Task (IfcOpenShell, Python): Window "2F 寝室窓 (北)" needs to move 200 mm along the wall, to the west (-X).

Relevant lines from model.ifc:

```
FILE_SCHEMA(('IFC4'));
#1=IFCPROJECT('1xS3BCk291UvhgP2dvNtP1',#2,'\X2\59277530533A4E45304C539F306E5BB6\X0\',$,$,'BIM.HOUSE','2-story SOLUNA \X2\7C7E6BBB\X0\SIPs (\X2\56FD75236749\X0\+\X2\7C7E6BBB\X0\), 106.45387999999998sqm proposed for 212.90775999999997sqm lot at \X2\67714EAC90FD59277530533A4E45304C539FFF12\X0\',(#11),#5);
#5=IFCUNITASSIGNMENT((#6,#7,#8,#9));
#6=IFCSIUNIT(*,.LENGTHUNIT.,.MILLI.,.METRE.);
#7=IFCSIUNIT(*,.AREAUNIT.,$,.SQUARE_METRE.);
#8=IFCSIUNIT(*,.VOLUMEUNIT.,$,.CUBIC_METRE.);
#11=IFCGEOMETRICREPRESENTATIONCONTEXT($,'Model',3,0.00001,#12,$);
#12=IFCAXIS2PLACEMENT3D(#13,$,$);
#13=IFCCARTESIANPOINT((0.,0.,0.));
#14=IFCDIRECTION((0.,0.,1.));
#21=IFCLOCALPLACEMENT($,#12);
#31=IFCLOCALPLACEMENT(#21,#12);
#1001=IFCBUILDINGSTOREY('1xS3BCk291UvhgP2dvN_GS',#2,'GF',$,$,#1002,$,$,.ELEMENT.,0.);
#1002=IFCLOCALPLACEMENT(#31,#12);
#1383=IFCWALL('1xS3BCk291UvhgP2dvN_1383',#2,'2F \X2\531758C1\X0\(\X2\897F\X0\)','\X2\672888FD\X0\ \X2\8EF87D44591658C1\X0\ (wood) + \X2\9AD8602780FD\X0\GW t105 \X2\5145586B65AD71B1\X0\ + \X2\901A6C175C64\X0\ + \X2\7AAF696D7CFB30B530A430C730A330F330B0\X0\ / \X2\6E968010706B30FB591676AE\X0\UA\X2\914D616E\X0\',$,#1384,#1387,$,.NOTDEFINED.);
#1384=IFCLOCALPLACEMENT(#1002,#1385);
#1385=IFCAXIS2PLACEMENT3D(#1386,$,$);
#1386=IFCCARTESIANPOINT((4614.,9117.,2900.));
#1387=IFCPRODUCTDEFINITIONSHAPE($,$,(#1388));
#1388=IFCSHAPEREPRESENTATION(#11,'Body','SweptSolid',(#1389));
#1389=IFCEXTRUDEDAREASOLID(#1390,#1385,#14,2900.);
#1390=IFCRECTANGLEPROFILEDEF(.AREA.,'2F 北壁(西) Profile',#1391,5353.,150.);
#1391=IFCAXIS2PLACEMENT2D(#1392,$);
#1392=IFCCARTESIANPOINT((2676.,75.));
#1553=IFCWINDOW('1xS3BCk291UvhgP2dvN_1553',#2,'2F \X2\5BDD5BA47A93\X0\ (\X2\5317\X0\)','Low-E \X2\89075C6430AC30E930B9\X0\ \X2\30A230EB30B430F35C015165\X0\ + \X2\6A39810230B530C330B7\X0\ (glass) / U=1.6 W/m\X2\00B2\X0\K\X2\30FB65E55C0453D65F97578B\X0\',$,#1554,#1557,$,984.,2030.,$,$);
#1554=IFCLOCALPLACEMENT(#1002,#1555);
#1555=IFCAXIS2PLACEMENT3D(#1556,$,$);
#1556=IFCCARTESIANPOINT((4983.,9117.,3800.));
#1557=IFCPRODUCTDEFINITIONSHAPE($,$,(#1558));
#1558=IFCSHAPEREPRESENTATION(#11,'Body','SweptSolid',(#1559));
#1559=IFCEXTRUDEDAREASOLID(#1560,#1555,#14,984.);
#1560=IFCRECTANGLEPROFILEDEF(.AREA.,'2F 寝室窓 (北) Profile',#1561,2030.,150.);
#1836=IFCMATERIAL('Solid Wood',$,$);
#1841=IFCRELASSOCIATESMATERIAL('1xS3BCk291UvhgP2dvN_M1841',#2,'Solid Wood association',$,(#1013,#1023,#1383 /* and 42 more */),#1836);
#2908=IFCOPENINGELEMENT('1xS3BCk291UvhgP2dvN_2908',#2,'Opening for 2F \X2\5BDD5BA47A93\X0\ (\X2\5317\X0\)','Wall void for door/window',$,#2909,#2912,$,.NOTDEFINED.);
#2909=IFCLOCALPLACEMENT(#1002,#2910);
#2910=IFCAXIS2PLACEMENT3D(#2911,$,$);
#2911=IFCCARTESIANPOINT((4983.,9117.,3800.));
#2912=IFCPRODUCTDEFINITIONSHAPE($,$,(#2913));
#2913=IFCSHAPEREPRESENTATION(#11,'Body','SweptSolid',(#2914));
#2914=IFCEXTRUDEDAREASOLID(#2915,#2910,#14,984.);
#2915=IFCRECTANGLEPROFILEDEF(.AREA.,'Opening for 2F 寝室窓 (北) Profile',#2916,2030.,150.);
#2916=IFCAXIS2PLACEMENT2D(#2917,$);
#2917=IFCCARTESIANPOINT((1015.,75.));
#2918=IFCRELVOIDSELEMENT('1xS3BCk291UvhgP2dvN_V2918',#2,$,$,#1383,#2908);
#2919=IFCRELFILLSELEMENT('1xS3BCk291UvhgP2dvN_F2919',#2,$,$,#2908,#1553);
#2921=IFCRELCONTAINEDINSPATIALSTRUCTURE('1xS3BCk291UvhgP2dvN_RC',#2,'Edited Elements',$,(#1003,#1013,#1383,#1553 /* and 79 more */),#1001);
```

```python
import ifcopenshell
import ifcopenshell.api.geometry
import ifcopenshell.util.placement
import ifcopenshell.util.unit

model = ifcopenshell.open("model.ifc")
unit_scale = ifcopenshell.util.unit.calculate_unit_scale(model)

window = model.by_guid("1xS3BCk291UvhgP2dvN_1553")
opening = window.FillsVoids[0].RelatingOpeningElement
wall = opening.VoidsElements[0].RelatingBuildingElement

wall_matrix = ifcopenshell.util.placement.get_local_placement(wall.ObjectPlacement)
shift = wall_matrix[:3, 0] * -0.2 / unit_scale
before = ifcopenshell.util.placement.get_local_placement(window.ObjectPlacement)[:3, 3].copy()

# The window is not placed relative to its opening, so move both.
for product in (opening, window):
    matrix = ifcopenshell.util.placement.get_local_placement(product.ObjectPlacement)
    matrix[:3, 3] += shift
    ifcopenshell.api.geometry.edit_object_placement(model, product=product, matrix=matrix, is_si=False)

after = ifcopenshell.util.placement.get_local_placement(window.ObjectPlacement)[:3, 3]
print("window moved by", (after - before).round(3) + 0.0)

model.write("model_updated.ifc")
```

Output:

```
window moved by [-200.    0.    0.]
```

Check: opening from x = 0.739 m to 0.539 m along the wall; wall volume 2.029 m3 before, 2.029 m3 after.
